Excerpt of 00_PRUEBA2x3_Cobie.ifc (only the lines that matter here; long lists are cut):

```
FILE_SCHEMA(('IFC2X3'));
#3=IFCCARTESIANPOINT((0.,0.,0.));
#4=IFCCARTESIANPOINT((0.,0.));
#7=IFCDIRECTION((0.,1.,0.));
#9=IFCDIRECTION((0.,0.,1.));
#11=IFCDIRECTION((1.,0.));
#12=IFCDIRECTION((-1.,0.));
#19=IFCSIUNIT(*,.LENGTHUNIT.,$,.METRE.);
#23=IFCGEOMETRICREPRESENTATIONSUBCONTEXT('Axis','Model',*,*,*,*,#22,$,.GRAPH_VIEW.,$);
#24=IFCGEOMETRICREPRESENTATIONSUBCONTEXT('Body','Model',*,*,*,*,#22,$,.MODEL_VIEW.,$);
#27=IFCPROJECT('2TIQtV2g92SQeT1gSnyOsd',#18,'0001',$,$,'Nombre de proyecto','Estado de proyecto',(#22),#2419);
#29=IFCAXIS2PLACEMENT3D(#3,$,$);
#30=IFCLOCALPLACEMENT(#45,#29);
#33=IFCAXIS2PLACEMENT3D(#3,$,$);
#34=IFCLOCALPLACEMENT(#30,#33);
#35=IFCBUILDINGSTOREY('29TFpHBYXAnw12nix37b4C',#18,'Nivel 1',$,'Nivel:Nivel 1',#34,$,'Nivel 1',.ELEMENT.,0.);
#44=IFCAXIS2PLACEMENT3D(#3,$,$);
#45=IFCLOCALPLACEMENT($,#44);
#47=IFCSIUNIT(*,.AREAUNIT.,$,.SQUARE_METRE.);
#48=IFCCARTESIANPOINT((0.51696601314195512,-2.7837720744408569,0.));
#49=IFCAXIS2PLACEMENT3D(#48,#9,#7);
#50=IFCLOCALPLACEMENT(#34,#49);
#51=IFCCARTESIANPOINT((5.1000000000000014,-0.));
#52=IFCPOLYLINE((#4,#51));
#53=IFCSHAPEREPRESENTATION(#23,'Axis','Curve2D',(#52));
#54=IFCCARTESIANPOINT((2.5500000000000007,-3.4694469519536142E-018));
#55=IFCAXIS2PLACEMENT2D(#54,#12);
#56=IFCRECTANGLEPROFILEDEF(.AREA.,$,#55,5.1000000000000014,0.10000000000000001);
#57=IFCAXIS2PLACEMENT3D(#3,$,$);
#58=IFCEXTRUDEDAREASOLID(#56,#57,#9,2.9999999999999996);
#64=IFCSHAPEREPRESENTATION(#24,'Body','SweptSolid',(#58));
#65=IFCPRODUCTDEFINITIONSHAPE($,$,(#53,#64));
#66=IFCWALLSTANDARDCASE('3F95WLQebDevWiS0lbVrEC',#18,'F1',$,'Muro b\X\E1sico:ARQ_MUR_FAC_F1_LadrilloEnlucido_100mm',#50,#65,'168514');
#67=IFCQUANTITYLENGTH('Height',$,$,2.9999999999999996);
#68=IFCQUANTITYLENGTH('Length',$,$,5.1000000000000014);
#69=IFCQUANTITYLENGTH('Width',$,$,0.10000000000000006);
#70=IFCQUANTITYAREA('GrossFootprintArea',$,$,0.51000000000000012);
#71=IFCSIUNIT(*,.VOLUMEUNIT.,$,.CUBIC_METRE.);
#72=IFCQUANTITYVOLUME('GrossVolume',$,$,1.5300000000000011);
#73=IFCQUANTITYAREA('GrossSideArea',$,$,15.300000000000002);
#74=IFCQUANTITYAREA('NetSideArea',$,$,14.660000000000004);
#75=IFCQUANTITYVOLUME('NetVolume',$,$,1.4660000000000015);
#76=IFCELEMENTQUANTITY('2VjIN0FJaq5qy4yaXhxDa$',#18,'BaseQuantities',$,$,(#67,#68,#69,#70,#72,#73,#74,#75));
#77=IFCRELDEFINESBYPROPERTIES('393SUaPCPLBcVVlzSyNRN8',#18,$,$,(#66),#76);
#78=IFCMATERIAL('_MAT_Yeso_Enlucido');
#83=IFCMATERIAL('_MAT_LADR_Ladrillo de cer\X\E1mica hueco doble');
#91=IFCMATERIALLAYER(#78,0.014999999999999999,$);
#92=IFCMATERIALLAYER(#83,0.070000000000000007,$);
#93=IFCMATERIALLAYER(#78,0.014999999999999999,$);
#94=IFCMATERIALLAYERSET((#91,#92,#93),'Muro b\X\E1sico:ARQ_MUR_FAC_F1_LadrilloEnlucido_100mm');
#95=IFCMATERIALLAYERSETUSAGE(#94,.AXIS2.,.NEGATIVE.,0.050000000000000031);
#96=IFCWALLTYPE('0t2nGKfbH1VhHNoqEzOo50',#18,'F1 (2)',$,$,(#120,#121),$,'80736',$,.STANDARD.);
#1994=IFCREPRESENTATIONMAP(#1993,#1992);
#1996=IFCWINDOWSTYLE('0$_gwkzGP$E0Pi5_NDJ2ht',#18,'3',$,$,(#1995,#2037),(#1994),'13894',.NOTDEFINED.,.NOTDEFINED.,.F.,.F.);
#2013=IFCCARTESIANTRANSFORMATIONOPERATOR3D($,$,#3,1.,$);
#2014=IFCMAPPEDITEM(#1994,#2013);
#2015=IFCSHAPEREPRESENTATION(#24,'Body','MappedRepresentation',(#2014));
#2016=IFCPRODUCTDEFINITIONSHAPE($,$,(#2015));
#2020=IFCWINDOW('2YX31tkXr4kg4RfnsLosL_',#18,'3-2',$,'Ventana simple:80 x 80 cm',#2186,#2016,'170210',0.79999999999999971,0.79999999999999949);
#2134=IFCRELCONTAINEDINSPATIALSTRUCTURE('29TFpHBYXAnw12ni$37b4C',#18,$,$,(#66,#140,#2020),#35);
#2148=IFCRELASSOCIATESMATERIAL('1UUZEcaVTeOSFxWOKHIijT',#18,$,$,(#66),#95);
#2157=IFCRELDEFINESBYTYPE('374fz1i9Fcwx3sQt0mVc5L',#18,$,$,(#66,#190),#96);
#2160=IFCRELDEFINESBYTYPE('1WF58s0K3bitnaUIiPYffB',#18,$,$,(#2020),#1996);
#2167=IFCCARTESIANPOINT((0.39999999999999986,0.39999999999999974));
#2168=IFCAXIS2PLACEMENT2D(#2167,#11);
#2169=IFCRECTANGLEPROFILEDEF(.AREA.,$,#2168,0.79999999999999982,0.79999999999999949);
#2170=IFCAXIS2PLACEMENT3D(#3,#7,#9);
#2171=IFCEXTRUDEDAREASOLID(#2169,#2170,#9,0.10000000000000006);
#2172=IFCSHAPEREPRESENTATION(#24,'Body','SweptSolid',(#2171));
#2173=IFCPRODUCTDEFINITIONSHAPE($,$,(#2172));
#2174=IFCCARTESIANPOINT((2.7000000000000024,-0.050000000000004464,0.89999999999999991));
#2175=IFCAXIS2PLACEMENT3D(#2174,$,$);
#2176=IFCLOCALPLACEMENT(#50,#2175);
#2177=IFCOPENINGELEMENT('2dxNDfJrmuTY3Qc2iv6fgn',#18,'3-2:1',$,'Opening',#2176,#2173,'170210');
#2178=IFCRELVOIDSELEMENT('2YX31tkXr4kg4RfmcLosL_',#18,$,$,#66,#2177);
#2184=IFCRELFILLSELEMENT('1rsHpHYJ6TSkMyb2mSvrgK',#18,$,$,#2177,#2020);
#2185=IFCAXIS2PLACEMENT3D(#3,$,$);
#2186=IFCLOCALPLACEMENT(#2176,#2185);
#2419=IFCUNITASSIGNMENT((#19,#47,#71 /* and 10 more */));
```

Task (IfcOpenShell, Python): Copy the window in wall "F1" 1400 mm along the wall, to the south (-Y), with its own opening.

```python
import ifcopenshell
import ifcopenshell.api.feature
import ifcopenshell.api.geometry
import ifcopenshell.api.pset
import ifcopenshell.api.root
import ifcopenshell.geom
import ifcopenshell.util.element
import ifcopenshell.util.placement
import ifcopenshell.util.shape
import ifcopenshell.util.unit

model = ifcopenshell.open("00_PRUEBA2x3_Cobie.ifc")
unit_scale = ifcopenshell.util.unit.calculate_unit_scale(model)
area_scale = ifcopenshell.util.unit.calculate_unit_scale(model, "AREAUNIT")
volume_scale = ifcopenshell.util.unit.calculate_unit_scale(model, "VOLUMEUNIT")
settings = ifcopenshell.geom.settings()


def volume(element):
    """Net volume in cubic metres, openings subtracted."""
    shape = ifcopenshell.geom.create_shape(settings, element)
    return ifcopenshell.util.shape.get_volume(shape.geometry)


def reuse_history(source, copy):
    """copy_class also copies each property set's owner history, people and application; keep the originals."""
    for rel in copy.IsDefinedBy:
        if rel.is_a("IfcRelDefinesByProperties") and (history := rel.RelatingPropertyDefinition.OwnerHistory):
            rel.RelatingPropertyDefinition.OwnerHistory = source.OwnerHistory
            ifcopenshell.util.element.remove_deep2(model, history)


window = model.by_guid("2YX31tkXr4kg4RfnsLosL_")
opening = window.FillsVoids[0].RelatingOpeningElement
wall = opening.VoidsElements[0].RelatingBuildingElement
before = volume(wall)
shift = ifcopenshell.util.placement.get_local_placement(wall.ObjectPlacement)[:3, 0] * -1.4 / unit_scale

# copy_class copies the void relationship, type, container and properties, but no geometry.
new_opening = ifcopenshell.api.root.copy_class(model, product=opening)
new_opening.Representation = ifcopenshell.util.element.copy_deep(
    model, opening.Representation, exclude=["IfcGeometricRepresentationContext", "IfcRepresentationMap"]
)
new_opening.Tag = None
reuse_history(opening, new_opening)
new_window = ifcopenshell.api.root.copy_class(model, product=window)
new_window.Representation = ifcopenshell.util.element.copy_deep(
    model, window.Representation, exclude=["IfcGeometricRepresentationContext", "IfcRepresentationMap"]
)
new_window.Tag = None
reuse_history(window, new_window)
fills = ifcopenshell.api.feature.add_filling(model, opening=new_opening, element=new_window)
fills.OwnerHistory = new_window.OwnerHistory  # required in IFC2X3

for old, new in ((opening, new_opening), (window, new_window)):
    matrix = ifcopenshell.util.placement.get_local_placement(old.ObjectPlacement)
    matrix[:3, 3] += shift
    ifcopenshell.api.geometry.edit_object_placement(model, product=new, matrix=matrix, is_si=False)

after = volume(wall)
thickness = 0.1  # wall thickness in metres

# Update the wall's stored quantities.
qto = model.by_id(ifcopenshell.util.element.get_pset(wall, "BaseQuantities", should_inherit=False)["id"])
ifcopenshell.api.pset.edit_qto(model, qto=qto, properties={
    "NetSideArea": after / thickness / area_scale,
    "NetVolume": after / volume_scale,
})

print(f"wall volume {before:.3f} -> {after:.3f} m3")

model.write("00_PRUEBA2x3_Cobie_v2.ifc")
```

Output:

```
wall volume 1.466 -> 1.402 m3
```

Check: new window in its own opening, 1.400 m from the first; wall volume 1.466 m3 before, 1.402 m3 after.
